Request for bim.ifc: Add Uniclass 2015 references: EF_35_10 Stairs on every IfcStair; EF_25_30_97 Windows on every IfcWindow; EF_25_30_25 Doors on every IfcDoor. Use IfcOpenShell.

First a look at what the model holds.

```python
import ifcopenshell

model = ifcopenshell.open("bim.ifc")
print(model.schema)
print("classifications:", [c.Name for c in model.by_type("IfcClassification")])
for ifc_class in ("IfcDoor", "IfcRoof", "IfcStair", "IfcWall", "IfcWindow"):
    print(ifc_class, len(model.by_type(ifc_class)))
```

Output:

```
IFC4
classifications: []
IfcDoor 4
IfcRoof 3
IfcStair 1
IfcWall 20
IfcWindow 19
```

```python
import ifcopenshell
import ifcopenshell.api.classification

model = ifcopenshell.open("bim.ifc")

system = ifcopenshell.api.classification.add_classification(model, classification="Uniclass 2015")

codes = {
    "IfcStair": ("EF_35_10", "Stairs"),
    "IfcWindow": ("EF_25_30_97", "Windows"),
    "IfcDoor": ("EF_25_30_25", "Doors"),
}
for ifc_class, (code, name) in codes.items():
    products = model.by_type(ifc_class)
    ifcopenshell.api.classification.add_reference(
        model, products=products, classification=system, identification=code, name=name
    )
    print(code, len(products))

model.write("bim_edited.ifc")
```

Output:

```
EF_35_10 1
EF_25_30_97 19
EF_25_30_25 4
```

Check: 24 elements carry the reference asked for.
